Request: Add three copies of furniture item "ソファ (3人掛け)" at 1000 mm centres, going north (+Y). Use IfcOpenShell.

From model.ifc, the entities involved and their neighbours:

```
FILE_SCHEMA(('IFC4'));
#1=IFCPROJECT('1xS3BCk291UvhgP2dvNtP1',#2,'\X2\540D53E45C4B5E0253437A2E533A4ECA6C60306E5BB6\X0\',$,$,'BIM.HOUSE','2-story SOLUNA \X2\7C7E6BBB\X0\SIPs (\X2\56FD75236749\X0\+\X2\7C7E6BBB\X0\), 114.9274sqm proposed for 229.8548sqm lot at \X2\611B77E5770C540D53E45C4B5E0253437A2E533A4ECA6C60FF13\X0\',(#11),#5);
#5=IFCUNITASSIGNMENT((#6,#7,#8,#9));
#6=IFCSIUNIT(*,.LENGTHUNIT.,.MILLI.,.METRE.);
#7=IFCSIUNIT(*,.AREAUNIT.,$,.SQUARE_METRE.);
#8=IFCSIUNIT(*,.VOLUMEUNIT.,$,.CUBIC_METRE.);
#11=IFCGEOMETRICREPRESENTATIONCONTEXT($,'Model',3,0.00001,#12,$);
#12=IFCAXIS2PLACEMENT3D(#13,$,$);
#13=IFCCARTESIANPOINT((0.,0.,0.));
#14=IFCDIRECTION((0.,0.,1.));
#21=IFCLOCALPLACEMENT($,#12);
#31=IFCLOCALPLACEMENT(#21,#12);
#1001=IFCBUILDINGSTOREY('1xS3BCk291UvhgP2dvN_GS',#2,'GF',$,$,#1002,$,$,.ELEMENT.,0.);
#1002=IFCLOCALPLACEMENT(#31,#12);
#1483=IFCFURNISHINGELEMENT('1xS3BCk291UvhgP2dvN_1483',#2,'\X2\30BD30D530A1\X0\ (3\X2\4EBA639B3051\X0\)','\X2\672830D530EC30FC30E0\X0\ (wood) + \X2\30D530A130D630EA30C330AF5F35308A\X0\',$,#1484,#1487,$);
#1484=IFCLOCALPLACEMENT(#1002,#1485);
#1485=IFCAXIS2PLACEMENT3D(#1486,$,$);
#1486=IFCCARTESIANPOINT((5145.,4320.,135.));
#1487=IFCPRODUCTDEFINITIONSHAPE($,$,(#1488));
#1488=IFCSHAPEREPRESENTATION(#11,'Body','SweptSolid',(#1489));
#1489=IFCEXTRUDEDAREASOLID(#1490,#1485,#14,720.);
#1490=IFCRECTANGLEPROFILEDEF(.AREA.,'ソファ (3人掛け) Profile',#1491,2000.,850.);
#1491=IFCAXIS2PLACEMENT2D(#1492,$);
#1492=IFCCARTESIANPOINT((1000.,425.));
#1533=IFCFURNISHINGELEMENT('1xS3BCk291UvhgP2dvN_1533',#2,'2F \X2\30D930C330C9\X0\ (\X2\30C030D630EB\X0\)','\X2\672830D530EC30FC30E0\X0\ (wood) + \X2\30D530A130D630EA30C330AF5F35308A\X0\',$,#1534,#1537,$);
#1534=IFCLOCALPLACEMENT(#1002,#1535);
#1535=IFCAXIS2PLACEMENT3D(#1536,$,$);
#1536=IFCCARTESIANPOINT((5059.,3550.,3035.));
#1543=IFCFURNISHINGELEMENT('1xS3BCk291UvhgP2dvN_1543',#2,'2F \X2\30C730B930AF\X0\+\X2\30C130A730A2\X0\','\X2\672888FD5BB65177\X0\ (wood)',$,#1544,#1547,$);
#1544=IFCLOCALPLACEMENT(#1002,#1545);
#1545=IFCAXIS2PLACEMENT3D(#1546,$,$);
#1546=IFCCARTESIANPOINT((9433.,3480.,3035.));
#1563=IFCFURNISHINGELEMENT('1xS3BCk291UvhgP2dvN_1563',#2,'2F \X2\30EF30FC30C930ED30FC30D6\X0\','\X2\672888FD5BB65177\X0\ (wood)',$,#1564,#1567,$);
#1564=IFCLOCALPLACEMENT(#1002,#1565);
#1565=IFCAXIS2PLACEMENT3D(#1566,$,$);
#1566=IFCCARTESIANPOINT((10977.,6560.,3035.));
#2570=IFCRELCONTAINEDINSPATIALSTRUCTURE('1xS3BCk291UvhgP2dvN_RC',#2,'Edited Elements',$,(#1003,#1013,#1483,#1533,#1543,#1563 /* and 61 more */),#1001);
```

```python
import numpy as np
import ifcopenshell
import ifcopenshell.api.geometry
import ifcopenshell.api.root
import ifcopenshell.util.element
import ifcopenshell.util.placement

model = ifcopenshell.open("model.ifc")


def reuse_history(source, copy):
    """copy_class also copies each property set's owner history, people and application; keep the originals."""
    for rel in copy.IsDefinedBy:
        if rel.is_a("IfcRelDefinesByProperties") and (history := rel.RelatingPropertyDefinition.OwnerHistory):
            rel.RelatingPropertyDefinition.OwnerHistory = source.OwnerHistory
            ifcopenshell.util.element.remove_deep2(model, history)


source = model.by_guid("1xS3BCk291UvhgP2dvN_1483")
base = ifcopenshell.util.placement.get_local_placement(source.ObjectPlacement)
step = np.array([0.0, 1.0, 0.0]) * 1000.0

for i in range(1, 4):
    copy = ifcopenshell.api.root.copy_class(model, product=source)
    copy.Representation = ifcopenshell.util.element.copy_deep(
        model, source.Representation, exclude=["IfcGeometricRepresentationContext", "IfcRepresentationMap"]
    )
    reuse_history(source, copy)
    matrix = base.copy()
    matrix[:3, 3] += i * step
    print("added at", matrix[:3, 3].round(3) + 0.0)
    ifcopenshell.api.geometry.edit_object_placement(model, product=copy, matrix=matrix, is_si=False)

model.write("model-out.ifc")
```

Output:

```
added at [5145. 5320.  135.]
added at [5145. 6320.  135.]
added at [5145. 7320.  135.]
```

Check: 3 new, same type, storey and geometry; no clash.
